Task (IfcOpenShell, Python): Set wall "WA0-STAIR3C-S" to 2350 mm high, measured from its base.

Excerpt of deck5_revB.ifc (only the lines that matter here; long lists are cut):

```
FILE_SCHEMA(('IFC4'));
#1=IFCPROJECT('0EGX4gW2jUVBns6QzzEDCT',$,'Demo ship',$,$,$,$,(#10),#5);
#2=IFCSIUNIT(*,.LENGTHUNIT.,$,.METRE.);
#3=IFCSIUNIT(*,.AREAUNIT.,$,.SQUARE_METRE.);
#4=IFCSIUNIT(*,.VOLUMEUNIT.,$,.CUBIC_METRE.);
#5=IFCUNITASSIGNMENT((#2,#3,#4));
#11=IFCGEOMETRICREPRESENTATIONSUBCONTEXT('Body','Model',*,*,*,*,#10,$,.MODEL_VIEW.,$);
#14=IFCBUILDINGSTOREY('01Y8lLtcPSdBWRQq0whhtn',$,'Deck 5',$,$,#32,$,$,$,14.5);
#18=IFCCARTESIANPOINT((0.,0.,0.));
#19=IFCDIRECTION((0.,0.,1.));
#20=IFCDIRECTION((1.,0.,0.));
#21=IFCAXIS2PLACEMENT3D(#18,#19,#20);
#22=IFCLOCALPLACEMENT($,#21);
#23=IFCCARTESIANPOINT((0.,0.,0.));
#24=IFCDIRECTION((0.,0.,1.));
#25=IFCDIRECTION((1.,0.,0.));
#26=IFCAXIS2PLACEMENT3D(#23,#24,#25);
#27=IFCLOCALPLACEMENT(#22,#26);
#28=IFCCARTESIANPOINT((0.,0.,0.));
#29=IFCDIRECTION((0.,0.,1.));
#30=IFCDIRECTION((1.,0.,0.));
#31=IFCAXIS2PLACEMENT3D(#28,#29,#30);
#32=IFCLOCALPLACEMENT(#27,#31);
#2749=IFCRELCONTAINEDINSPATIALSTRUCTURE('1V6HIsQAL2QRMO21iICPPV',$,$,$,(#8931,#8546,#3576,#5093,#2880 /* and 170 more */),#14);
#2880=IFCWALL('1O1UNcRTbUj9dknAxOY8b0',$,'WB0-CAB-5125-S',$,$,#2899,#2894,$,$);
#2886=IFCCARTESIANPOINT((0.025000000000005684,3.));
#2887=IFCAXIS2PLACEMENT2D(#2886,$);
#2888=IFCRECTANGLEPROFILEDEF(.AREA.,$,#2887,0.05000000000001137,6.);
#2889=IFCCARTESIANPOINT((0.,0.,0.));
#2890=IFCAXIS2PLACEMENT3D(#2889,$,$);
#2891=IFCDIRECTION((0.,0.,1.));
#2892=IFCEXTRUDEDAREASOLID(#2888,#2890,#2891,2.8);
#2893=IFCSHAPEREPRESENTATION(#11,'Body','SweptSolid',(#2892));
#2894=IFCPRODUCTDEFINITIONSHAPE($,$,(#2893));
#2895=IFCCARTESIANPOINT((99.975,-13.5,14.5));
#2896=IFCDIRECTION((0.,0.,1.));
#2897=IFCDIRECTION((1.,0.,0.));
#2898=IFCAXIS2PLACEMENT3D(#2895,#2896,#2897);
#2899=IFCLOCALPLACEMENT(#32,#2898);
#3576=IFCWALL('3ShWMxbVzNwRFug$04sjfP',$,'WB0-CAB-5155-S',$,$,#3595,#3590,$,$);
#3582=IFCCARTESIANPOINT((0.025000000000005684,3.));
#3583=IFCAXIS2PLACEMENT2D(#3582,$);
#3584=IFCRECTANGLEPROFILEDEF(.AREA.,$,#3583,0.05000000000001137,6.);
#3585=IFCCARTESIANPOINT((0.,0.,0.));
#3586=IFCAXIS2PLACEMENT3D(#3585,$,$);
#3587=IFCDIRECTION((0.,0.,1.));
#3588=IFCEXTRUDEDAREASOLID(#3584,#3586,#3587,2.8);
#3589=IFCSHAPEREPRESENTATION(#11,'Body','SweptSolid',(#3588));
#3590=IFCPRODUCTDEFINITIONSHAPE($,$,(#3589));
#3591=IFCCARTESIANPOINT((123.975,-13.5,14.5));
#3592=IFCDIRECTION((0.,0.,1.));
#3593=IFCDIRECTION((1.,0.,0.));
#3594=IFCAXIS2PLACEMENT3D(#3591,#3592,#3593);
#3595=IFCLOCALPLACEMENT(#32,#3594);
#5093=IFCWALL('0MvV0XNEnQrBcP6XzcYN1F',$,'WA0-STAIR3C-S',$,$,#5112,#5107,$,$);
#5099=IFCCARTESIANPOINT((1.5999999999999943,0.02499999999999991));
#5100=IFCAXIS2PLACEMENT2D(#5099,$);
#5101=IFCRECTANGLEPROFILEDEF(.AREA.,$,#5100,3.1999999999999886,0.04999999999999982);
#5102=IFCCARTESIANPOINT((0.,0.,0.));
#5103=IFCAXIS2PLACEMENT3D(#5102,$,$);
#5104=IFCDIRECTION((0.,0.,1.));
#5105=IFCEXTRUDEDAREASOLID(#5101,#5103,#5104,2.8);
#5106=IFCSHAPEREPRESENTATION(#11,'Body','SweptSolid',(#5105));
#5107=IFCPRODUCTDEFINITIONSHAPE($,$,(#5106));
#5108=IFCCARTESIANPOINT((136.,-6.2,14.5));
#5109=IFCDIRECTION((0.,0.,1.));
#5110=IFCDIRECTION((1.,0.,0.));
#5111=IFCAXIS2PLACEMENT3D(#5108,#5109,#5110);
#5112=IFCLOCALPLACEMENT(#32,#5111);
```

```python
import ifcopenshell
import ifcopenshell.geom
import ifcopenshell.util.representation
import ifcopenshell.util.shape

model = ifcopenshell.open("deck5_revB.ifc")
settings = ifcopenshell.geom.settings()


def volume(element):
    """Net volume in cubic metres, openings subtracted."""
    shape = ifcopenshell.geom.create_shape(settings, element)
    return ifcopenshell.util.shape.get_volume(shape.geometry)


wall = model.by_guid("0MvV0XNEnQrBcP6XzcYN1F")
before = volume(wall)

body = ifcopenshell.util.representation.get_representation(wall, "Model", "Body")
solid = body.Items[0]
old_height = solid.Depth
solid.Depth = 2.35
after = volume(wall)

print(f"height {old_height:g} -> {solid.Depth:g}, volume {before:.3f} -> {after:.3f} m3")

model.write("deck5_revB_rev.ifc")
```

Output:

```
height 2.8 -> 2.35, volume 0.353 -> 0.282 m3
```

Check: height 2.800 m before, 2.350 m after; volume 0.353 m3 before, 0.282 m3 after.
